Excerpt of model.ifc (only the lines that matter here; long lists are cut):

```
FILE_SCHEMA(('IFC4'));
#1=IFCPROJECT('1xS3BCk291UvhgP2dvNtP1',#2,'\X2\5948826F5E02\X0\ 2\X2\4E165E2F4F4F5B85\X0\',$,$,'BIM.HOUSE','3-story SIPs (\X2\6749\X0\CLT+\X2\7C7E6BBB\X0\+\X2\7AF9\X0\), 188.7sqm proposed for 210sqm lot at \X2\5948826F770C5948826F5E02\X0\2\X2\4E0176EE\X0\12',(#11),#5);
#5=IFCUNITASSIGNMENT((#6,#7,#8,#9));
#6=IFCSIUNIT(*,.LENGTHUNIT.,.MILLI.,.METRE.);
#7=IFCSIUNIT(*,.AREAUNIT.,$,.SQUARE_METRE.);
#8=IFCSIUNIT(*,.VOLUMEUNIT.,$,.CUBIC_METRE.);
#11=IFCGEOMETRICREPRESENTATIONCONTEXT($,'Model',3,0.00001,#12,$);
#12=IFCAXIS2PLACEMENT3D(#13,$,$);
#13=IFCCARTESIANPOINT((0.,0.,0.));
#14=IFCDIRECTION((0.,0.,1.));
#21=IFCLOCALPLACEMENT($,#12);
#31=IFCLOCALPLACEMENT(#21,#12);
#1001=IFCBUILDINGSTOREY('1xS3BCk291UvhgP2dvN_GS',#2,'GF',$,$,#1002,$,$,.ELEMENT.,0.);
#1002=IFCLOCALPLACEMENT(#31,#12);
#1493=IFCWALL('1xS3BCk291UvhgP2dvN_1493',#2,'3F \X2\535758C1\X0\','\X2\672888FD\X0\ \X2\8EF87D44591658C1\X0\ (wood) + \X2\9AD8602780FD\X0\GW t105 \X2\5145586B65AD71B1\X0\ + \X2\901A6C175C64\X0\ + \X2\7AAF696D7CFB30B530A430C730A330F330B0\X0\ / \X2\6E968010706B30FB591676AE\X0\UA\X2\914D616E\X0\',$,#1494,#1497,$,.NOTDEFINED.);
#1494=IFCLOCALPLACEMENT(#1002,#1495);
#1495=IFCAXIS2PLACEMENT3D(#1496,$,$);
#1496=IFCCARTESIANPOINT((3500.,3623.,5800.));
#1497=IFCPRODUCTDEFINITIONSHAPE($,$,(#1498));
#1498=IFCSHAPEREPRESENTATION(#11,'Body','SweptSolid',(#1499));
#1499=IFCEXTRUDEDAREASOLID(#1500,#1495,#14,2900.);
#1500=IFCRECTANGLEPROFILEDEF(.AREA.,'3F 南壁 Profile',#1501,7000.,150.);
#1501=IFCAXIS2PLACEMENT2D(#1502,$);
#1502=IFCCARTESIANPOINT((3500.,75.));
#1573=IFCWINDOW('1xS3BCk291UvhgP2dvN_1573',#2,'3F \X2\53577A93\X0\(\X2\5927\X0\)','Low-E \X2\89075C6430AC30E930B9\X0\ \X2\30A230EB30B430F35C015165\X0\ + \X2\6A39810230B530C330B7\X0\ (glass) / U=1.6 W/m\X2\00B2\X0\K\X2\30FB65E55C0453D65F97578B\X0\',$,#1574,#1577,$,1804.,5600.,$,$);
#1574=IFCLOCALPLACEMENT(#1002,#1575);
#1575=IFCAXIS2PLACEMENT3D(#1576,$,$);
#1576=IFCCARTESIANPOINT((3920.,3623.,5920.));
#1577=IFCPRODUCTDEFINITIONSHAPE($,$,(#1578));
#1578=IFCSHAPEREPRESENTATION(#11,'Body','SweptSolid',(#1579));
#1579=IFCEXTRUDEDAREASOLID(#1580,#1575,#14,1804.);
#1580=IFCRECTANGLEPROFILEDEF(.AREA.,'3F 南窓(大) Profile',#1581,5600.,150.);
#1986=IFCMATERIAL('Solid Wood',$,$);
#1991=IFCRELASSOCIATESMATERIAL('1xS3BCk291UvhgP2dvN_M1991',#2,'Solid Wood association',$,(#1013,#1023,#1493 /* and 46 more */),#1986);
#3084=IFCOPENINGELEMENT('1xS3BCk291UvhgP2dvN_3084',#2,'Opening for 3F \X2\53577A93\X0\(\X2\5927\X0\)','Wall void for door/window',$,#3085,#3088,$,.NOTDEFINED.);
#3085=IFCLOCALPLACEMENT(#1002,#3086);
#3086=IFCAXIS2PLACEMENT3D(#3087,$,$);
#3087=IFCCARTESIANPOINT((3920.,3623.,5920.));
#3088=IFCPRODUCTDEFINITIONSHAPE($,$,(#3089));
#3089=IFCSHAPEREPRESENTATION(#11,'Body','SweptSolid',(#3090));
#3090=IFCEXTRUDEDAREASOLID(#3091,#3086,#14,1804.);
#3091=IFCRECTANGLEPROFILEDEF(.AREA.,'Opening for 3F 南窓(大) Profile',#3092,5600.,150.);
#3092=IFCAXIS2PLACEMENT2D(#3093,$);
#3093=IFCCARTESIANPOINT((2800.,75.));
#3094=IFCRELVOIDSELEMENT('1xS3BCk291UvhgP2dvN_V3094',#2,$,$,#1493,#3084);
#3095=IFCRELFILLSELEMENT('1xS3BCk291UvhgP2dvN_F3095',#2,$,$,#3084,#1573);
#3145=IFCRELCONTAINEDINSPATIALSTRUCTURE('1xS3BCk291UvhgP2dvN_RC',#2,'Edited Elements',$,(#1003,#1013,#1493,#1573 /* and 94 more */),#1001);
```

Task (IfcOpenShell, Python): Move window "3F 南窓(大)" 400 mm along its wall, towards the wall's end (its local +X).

```python
import ifcopenshell
import ifcopenshell.api.geometry
import ifcopenshell.util.placement
import ifcopenshell.util.unit

model = ifcopenshell.open("model.ifc")
unit_scale = ifcopenshell.util.unit.calculate_unit_scale(model)

window = model.by_guid("1xS3BCk291UvhgP2dvN_1573")
opening = window.FillsVoids[0].RelatingOpeningElement
wall = opening.VoidsElements[0].RelatingBuildingElement

wall_matrix = ifcopenshell.util.placement.get_local_placement(wall.ObjectPlacement)
shift = wall_matrix[:3, 0] * 0.4 / unit_scale
before = ifcopenshell.util.placement.get_local_placement(window.ObjectPlacement)[:3, 3].copy()

# The window is not placed relative to its opening, so move both.
for product in (opening, window):
    matrix = ifcopenshell.util.placement.get_local_placement(product.ObjectPlacement)
    matrix[:3, 3] += shift
    ifcopenshell.api.geometry.edit_object_placement(model, product=product, matrix=matrix, is_si=False)

after = ifcopenshell.util.placement.get_local_placement(window.ObjectPlacement)[:3, 3]
print("window moved by", (after - before).round(3) + 0.0)

model.write("model_rev.ifc")
```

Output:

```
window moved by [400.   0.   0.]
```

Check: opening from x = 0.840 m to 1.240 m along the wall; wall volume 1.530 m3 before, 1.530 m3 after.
